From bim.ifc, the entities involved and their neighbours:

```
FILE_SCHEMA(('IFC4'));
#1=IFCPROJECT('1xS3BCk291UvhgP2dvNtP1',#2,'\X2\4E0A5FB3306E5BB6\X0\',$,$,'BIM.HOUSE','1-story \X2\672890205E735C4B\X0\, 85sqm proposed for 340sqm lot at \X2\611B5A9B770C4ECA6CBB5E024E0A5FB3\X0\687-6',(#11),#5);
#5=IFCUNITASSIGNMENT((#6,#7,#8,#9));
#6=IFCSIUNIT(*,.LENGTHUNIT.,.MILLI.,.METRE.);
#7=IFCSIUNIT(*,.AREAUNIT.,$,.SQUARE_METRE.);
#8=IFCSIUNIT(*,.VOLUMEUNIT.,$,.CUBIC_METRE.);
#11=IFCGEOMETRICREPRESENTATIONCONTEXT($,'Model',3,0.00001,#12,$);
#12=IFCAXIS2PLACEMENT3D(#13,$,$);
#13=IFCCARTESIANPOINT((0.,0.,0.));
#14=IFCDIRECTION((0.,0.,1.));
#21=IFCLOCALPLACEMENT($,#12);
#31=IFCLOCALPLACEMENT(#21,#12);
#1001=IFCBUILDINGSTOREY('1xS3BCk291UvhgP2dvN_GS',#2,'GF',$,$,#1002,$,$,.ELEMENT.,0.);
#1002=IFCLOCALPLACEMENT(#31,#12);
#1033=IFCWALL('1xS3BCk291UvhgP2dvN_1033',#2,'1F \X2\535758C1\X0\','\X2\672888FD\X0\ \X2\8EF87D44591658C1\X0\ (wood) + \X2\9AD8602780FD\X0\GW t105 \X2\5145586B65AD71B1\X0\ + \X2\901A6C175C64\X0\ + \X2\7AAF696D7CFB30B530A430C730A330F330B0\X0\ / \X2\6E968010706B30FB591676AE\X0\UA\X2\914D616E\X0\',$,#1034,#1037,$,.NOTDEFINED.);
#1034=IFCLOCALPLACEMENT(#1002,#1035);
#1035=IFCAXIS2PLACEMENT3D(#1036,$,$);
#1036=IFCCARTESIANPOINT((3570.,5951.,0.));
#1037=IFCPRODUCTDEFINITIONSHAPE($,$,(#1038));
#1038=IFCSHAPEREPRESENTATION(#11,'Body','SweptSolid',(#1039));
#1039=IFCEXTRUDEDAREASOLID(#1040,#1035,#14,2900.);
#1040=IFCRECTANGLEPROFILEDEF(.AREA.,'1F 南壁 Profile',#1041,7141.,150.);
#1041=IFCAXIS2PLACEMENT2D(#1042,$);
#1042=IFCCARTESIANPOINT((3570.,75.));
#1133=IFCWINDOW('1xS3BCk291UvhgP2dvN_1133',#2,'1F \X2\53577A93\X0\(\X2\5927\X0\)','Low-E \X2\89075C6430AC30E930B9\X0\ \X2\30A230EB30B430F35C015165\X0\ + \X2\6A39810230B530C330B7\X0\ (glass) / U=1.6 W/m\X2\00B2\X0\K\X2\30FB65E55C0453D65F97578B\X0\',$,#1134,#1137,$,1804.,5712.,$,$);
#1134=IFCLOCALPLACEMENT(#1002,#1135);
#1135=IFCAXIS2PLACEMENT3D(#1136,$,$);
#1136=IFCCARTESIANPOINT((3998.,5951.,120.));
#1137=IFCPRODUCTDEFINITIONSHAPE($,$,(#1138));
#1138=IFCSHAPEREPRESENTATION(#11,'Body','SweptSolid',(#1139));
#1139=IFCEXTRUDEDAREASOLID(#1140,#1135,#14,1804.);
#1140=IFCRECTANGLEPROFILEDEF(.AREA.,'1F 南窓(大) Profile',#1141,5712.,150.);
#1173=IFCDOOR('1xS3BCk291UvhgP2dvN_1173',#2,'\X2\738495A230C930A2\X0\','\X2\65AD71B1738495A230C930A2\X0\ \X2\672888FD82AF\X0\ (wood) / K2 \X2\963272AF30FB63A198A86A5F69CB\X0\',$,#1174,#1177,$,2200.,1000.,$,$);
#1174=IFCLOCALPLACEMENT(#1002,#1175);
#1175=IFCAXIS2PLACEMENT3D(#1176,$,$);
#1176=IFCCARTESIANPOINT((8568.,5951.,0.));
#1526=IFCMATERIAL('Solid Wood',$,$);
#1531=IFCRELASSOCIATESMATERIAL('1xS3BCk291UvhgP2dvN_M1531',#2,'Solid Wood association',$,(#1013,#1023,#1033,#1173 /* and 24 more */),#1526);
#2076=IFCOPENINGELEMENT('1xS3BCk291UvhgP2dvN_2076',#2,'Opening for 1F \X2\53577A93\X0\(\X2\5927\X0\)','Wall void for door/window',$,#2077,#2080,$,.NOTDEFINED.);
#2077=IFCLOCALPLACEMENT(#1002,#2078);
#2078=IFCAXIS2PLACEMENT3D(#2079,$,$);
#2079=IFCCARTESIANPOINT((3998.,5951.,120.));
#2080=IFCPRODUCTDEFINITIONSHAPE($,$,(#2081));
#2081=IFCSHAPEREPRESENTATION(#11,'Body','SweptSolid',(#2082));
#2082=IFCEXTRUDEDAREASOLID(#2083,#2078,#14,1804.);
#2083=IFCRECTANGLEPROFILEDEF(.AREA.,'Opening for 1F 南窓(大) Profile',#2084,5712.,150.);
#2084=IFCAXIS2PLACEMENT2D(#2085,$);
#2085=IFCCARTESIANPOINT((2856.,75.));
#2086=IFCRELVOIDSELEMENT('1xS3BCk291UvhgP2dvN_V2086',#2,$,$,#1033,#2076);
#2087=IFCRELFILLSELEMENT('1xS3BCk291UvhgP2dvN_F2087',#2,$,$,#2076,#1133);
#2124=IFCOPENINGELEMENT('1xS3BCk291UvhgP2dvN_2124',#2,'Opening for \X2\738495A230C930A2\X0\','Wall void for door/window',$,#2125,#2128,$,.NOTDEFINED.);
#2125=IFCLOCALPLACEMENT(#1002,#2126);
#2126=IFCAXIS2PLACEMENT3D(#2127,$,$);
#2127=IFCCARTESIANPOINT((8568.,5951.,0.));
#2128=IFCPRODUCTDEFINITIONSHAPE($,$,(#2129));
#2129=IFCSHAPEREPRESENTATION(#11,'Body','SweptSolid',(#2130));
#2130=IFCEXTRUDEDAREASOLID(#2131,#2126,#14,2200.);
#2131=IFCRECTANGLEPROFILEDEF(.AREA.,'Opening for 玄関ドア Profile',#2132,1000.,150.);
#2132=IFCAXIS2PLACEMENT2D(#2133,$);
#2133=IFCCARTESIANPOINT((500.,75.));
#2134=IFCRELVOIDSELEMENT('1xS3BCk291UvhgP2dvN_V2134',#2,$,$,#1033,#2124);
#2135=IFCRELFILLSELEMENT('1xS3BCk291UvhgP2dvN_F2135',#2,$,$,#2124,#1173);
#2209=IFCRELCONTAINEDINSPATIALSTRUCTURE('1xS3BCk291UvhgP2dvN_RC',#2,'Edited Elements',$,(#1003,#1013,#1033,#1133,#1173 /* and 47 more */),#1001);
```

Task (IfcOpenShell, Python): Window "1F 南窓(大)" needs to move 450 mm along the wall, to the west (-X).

```python
import ifcopenshell
import ifcopenshell.api.geometry
import ifcopenshell.util.placement

model = ifcopenshell.open("bim.ifc")

window = model.by_id(1133)
opening = window.FillsVoids[0].RelatingOpeningElement
wall = opening.VoidsElements[0].RelatingBuildingElement

wall_matrix = ifcopenshell.util.placement.get_local_placement(wall.ObjectPlacement)
shift = wall_matrix[:3, 0] * -450.0
before = ifcopenshell.util.placement.get_local_placement(window.ObjectPlacement)[:3, 3].copy()

# The window is not placed relative to its opening, so move both.
for product in (opening, window):
    matrix = ifcopenshell.util.placement.get_local_placement(product.ObjectPlacement)
    matrix[:3, 3] += shift
    ifcopenshell.api.geometry.edit_object_placement(model, product=product, matrix=matrix, is_si=False)

after = ifcopenshell.util.placement.get_local_placement(window.ObjectPlacement)[:3, 3]
print("window moved by", (after - before).round(3) + 0.0)

model.write("bim-out.ifc")
```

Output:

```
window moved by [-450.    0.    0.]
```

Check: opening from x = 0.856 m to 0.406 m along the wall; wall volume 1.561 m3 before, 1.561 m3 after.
